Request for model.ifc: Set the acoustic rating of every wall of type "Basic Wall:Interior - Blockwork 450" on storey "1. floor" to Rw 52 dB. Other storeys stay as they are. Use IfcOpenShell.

First a look at what the model holds.

```python
import ifcopenshell
import ifcopenshell.util.element

model = ifcopenshell.open("model.ifc")
print(model.schema)
storey = next(s for s in model.by_type("IfcBuildingStorey") if s.Name == "1. floor")
walls = [e for e in ifcopenshell.util.element.get_decomposition(storey) if e.is_a("IfcWall")]
seen = {}
for e in walls:
    element_type = ifcopenshell.util.element.get_type(e)
    key = (element_type.Name if element_type != e and element_type else None, ifcopenshell.util.element.get_pset(e, "Pset_WallCommon", "AcousticRating"))
    seen[key] = seen.get(key, 0) + 1
for (name, value), count in sorted(seen.items(), key=str):
    print(count, "x", name, "|", value)
```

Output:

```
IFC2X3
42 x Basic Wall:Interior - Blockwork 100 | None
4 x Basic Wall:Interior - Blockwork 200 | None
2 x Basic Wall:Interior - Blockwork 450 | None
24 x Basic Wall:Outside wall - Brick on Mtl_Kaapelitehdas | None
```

```python
import ifcopenshell
import ifcopenshell.api.pset
import ifcopenshell.util.element

model = ifcopenshell.open("model.ifc")

storey = next(s for s in model.by_type("IfcBuildingStorey") if s.Name == "1. floor")
walls = [e for e in ifcopenshell.util.element.get_decomposition(storey) if e.is_a("IfcWall")]

count = 0
for e in walls:
    element_type = ifcopenshell.util.element.get_type(e)
    if element_type in (None, e) or element_type.Name != "Basic Wall:Interior - Blockwork 450":
        continue
    # add_pset returns the element's existing set when there is one.
    pset = ifcopenshell.api.pset.add_pset(model, product=e, name="Pset_WallCommon")
    ifcopenshell.api.pset.edit_pset(model, pset=pset, properties={"AcousticRating": "Rw 52 dB"})
    count += 1

print(count, "walls updated")

model.write("model_v2.ifc")
```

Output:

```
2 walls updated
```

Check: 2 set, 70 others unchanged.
